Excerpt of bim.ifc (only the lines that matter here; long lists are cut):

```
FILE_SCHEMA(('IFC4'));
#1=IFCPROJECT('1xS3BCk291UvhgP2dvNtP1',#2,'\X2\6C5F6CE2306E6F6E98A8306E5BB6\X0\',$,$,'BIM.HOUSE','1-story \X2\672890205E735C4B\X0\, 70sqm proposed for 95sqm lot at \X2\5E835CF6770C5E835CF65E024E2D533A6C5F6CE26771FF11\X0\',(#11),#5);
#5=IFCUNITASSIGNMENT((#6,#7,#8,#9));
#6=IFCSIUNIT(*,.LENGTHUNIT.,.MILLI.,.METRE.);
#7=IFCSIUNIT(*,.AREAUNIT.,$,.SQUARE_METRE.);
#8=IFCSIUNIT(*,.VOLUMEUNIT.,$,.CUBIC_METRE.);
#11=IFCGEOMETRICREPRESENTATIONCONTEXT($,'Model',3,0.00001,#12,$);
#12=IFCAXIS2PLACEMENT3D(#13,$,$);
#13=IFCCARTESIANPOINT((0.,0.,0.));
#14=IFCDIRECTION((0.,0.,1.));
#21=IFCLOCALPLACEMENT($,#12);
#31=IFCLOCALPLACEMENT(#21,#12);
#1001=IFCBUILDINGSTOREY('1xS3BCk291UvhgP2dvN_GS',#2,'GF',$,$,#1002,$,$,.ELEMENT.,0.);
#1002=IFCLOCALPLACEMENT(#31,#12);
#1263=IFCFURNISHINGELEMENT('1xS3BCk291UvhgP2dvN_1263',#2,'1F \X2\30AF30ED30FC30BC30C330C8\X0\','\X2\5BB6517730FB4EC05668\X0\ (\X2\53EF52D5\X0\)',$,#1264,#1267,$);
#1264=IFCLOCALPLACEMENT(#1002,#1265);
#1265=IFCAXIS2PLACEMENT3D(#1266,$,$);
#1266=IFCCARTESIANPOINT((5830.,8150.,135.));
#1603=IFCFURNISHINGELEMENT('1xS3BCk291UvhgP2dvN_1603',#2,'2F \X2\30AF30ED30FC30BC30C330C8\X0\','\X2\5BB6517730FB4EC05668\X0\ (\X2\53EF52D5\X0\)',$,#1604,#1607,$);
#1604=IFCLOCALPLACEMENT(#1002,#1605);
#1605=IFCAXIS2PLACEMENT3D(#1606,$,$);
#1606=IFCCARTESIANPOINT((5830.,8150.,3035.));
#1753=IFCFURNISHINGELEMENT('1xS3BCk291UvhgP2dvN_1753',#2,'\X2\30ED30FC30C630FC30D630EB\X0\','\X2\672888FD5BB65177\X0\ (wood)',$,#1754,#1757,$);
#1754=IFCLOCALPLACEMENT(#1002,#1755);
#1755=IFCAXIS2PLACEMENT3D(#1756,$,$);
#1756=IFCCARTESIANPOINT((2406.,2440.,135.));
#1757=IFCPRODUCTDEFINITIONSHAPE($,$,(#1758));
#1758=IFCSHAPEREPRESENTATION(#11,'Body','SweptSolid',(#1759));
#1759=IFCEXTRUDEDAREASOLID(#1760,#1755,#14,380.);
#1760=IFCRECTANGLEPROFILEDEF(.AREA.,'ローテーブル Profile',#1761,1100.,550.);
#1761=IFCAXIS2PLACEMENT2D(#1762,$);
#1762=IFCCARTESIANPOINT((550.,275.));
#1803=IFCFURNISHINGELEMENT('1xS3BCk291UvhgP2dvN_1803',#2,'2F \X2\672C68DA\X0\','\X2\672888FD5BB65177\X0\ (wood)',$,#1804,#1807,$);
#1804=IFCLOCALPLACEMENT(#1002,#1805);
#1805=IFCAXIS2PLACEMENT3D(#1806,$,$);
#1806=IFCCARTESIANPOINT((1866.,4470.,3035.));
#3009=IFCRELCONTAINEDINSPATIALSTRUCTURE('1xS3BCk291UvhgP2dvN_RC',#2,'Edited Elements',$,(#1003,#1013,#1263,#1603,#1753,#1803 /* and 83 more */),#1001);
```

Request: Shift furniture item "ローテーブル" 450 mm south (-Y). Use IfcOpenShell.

```python
import ifcopenshell
import ifcopenshell.api.geometry
import ifcopenshell.util.placement
import ifcopenshell.util.unit

model = ifcopenshell.open("bim.ifc")
unit_scale = ifcopenshell.util.unit.calculate_unit_scale(model)

item = model.by_guid("1xS3BCk291UvhgP2dvN_1753")
matrix = ifcopenshell.util.placement.get_local_placement(item.ObjectPlacement)
matrix[1, 3] -= 0.45 / unit_scale
ifcopenshell.api.geometry.edit_object_placement(model, product=item, matrix=matrix, is_si=False)

print(ifcopenshell.util.placement.get_local_placement(item.ObjectPlacement).round(3) + 0.0)

model.write("bim_v2.ifc")
```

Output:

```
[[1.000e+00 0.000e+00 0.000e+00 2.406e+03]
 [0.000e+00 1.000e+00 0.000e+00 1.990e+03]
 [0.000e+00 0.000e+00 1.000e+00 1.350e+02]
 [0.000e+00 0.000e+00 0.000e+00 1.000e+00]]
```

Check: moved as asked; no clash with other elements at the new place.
